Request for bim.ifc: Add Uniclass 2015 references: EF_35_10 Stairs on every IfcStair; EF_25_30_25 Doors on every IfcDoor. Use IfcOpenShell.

First a look at what the model holds.

```python
import ifcopenshell

model = ifcopenshell.open("bim.ifc")
print(model.schema)
print("classifications:", [c.Name for c in model.by_type("IfcClassification")])
for ifc_class in ("IfcDoor", "IfcRoof", "IfcStair", "IfcWall", "IfcWindow"):
    print(ifc_class, len(model.by_type(ifc_class)))
```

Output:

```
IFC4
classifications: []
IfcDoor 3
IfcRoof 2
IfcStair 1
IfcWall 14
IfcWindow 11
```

```python
import ifcopenshell
import ifcopenshell.api.classification

model = ifcopenshell.open("bim.ifc")

system = ifcopenshell.api.classification.add_classification(model, classification="Uniclass 2015")

codes = {
    "IfcStair": ("EF_35_10", "Stairs"),
    "IfcDoor": ("EF_25_30_25", "Doors"),
}
for ifc_class, (code, name) in codes.items():
    products = model.by_type(ifc_class)
    ifcopenshell.api.classification.add_reference(
        model, products=products, classification=system, identification=code, name=name
    )
    print(code, len(products))

model.write("bim-out.ifc")
```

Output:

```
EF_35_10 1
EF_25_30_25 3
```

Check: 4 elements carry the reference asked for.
